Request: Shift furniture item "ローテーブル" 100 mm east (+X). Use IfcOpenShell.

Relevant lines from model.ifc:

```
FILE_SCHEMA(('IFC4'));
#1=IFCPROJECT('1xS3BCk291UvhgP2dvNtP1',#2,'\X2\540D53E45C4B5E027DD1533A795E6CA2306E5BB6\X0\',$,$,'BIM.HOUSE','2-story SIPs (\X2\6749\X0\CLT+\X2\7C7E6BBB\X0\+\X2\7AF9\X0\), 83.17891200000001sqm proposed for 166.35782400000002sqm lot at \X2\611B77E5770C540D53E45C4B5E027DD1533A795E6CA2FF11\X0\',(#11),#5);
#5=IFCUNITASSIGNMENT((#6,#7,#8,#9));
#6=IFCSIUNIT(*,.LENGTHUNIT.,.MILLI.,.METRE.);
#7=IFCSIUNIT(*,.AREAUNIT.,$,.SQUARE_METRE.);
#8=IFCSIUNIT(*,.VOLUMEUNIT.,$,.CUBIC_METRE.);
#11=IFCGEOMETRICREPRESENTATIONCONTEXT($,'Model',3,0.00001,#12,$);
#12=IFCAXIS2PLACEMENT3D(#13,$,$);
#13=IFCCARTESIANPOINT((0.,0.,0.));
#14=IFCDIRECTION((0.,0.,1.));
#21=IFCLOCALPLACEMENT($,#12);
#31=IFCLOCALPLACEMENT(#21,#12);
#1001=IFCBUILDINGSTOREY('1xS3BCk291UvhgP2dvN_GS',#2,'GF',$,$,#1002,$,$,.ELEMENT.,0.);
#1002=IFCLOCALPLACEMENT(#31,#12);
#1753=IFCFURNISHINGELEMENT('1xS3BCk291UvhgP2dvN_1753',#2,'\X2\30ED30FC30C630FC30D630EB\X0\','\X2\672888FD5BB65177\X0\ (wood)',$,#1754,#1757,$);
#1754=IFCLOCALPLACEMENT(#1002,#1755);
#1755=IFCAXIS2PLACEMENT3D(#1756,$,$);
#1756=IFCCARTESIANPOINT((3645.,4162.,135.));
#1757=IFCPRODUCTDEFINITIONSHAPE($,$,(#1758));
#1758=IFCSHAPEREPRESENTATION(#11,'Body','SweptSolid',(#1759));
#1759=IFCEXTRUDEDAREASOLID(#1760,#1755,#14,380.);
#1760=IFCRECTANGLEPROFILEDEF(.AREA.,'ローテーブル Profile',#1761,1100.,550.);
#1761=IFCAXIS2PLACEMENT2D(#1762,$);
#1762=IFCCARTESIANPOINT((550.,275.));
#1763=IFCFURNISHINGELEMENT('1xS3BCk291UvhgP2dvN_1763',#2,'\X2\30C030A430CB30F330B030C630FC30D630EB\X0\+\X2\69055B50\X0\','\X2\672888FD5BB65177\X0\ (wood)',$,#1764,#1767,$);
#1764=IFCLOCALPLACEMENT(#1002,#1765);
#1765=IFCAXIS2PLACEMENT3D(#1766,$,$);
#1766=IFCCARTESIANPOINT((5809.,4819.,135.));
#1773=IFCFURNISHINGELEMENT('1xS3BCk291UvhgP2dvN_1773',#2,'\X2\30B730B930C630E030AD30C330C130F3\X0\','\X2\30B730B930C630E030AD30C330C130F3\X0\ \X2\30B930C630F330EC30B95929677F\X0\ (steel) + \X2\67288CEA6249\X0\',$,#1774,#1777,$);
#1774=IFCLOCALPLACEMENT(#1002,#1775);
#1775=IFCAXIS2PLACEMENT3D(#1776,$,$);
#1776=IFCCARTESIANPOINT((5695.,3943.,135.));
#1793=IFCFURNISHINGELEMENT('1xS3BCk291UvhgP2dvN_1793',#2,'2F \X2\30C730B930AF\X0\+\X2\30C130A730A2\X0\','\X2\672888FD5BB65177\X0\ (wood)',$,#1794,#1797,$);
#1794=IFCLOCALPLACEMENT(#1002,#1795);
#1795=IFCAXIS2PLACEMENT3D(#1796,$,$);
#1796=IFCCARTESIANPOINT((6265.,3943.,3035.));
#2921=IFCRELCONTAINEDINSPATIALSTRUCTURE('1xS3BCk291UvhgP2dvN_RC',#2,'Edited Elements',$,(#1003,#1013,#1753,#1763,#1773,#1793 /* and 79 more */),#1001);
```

```python
import ifcopenshell
import ifcopenshell.api.geometry
import ifcopenshell.util.placement

model = ifcopenshell.open("model.ifc")

item = model.by_guid("1xS3BCk291UvhgP2dvN_1753")
matrix = ifcopenshell.util.placement.get_local_placement(item.ObjectPlacement)
matrix[0, 3] += 100.0
ifcopenshell.api.geometry.edit_object_placement(model, product=item, matrix=matrix, is_si=False)

print(ifcopenshell.util.placement.get_local_placement(item.ObjectPlacement).round(3) + 0.0)

model.write("model-out.ifc")
```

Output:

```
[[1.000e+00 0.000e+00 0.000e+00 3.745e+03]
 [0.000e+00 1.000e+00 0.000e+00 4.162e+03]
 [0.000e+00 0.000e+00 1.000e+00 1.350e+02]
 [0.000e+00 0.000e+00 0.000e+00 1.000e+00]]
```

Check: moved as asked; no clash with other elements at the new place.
